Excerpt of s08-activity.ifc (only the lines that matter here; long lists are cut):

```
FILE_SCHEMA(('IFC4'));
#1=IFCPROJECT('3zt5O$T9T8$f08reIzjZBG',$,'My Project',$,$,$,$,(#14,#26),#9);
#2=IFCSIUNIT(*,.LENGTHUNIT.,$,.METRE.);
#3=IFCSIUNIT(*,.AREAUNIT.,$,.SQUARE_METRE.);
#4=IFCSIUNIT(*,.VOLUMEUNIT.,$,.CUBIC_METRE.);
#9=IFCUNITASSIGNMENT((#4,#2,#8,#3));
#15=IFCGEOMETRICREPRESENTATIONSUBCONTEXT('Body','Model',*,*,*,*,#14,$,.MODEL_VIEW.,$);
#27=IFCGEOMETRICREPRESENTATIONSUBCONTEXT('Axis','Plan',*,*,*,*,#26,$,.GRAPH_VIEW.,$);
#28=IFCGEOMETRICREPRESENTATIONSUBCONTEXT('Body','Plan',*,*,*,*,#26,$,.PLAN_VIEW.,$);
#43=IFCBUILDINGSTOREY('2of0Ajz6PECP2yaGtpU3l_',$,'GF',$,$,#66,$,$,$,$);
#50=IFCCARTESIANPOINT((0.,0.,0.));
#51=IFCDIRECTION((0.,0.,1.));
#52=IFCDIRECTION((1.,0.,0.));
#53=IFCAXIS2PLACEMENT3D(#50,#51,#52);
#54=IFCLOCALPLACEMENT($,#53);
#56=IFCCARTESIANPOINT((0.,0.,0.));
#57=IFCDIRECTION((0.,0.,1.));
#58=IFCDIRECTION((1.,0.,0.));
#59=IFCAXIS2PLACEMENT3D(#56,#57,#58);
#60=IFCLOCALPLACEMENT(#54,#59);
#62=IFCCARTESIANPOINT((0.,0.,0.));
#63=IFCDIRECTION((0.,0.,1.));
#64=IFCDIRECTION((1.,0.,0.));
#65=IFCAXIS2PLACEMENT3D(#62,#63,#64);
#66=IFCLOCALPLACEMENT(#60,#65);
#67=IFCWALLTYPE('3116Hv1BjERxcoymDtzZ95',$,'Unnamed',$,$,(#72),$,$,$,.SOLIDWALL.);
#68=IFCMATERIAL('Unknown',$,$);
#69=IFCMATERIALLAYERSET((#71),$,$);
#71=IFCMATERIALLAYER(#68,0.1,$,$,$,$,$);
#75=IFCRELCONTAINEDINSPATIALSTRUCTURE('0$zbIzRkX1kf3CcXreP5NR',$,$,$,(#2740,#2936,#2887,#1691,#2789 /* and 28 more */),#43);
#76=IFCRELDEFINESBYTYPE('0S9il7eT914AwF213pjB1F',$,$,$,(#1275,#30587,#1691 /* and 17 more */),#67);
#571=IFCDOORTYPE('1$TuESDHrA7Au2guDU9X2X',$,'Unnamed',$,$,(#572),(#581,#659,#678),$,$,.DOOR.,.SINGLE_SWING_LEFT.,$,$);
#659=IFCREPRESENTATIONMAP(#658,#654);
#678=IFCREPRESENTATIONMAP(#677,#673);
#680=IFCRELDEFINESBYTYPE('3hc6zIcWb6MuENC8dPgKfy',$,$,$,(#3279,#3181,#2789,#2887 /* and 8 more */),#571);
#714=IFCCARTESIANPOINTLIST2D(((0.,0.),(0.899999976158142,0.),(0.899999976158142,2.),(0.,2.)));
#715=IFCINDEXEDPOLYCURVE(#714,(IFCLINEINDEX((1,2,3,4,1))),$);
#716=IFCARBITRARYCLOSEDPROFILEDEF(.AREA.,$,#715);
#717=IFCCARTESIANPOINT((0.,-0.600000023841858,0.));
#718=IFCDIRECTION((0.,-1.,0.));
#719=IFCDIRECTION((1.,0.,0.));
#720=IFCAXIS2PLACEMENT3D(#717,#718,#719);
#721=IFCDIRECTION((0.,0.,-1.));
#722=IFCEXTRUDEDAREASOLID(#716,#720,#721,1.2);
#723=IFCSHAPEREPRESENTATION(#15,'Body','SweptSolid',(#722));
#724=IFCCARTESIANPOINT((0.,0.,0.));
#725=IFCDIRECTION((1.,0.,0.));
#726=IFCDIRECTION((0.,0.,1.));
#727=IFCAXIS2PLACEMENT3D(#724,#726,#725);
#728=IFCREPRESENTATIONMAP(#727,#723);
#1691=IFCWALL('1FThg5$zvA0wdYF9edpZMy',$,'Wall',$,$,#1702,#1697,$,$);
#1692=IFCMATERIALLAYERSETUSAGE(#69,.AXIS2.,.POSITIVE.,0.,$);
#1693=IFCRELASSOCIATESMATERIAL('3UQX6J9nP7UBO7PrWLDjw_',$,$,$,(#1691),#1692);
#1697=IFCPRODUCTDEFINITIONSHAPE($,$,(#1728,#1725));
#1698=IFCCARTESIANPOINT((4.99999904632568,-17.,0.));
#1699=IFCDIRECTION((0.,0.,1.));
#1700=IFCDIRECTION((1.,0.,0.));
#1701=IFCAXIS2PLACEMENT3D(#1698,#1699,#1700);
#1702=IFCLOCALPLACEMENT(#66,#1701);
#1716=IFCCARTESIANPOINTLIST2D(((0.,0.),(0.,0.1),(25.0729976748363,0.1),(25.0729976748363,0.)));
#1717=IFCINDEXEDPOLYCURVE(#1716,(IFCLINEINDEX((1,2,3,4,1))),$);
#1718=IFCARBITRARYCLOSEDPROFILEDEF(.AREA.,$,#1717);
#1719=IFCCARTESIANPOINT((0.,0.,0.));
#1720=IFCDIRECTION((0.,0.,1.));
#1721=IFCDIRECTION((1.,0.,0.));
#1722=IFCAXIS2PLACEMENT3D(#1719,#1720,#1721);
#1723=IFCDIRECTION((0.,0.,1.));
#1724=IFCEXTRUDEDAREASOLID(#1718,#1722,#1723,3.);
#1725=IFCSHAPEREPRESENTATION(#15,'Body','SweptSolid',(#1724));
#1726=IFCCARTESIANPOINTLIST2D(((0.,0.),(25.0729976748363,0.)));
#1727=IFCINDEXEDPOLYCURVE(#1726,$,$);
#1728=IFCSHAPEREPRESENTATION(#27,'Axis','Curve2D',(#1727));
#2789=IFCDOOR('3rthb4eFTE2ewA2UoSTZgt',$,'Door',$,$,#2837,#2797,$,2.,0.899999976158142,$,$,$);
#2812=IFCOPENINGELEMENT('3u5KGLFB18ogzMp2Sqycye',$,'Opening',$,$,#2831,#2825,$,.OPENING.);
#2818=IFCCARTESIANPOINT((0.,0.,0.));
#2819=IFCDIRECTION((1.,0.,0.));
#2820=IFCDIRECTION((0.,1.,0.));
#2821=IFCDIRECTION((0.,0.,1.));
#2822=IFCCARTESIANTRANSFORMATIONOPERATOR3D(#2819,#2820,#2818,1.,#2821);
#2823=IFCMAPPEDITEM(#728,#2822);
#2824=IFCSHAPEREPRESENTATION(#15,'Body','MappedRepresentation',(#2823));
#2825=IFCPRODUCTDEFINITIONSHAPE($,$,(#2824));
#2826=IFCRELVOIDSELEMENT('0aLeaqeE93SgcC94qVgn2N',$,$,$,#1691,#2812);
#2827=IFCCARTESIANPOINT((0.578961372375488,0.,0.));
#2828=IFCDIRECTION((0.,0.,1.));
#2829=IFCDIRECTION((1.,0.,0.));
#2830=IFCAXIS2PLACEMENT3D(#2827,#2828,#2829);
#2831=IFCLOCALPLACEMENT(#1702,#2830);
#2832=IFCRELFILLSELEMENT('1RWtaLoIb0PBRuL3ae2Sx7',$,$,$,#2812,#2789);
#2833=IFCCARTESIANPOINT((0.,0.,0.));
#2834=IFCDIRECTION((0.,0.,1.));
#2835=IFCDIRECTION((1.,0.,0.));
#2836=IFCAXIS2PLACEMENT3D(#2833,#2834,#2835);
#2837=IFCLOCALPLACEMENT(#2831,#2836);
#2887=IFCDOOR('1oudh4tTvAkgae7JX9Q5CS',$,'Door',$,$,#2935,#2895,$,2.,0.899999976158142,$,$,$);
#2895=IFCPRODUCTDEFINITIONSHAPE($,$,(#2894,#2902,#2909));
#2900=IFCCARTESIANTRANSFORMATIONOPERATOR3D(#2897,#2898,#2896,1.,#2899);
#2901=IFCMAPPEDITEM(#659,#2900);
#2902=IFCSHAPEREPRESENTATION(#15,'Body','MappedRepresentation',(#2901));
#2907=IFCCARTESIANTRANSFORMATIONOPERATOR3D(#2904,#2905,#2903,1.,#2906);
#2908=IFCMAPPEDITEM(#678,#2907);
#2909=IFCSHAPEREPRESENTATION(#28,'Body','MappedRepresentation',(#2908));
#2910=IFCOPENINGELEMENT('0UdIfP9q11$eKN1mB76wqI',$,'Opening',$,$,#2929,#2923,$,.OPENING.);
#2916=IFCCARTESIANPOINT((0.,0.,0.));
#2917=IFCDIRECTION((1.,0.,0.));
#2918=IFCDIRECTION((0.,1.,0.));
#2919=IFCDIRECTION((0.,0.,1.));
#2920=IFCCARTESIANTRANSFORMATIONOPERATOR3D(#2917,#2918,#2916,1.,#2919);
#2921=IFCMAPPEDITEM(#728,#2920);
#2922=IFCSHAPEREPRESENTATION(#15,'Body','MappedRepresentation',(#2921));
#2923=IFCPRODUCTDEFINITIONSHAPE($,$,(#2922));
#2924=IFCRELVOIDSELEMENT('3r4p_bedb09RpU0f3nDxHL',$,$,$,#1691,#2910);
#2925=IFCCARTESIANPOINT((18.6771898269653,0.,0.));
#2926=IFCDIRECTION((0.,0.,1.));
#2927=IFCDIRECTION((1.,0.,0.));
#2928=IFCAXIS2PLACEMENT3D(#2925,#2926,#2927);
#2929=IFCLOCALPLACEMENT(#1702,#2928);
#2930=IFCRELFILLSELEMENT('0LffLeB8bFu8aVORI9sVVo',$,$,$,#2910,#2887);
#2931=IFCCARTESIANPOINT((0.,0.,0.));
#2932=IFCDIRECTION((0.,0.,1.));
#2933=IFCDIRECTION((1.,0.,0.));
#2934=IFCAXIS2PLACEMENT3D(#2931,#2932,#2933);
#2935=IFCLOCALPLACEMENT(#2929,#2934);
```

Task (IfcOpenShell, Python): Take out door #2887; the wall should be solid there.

```python
import ifcopenshell
import ifcopenshell.api.feature
import ifcopenshell.api.root
import ifcopenshell.geom
import ifcopenshell.util.shape

model = ifcopenshell.open("s08-activity.ifc")
settings = ifcopenshell.geom.settings()


def volume(element):
    """Net volume in cubic metres, openings subtracted."""
    shape = ifcopenshell.geom.create_shape(settings, element)
    return ifcopenshell.util.shape.get_volume(shape.geometry)


door = model.by_guid("1oudh4tTvAkgae7JX9Q5CS")
opening = door.FillsVoids[0].RelatingOpeningElement
wall = opening.VoidsElements[0].RelatingBuildingElement
before = volume(wall)

ifcopenshell.api.root.remove_product(model, product=door)
ifcopenshell.api.feature.remove_feature(model, feature=opening)

after = volume(wall)

print(f"wall volume {before:.3f} -> {after:.3f} m3")

model.write("s08-activity_rev.ifc")
```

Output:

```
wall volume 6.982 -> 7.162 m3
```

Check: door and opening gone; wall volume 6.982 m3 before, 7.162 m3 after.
